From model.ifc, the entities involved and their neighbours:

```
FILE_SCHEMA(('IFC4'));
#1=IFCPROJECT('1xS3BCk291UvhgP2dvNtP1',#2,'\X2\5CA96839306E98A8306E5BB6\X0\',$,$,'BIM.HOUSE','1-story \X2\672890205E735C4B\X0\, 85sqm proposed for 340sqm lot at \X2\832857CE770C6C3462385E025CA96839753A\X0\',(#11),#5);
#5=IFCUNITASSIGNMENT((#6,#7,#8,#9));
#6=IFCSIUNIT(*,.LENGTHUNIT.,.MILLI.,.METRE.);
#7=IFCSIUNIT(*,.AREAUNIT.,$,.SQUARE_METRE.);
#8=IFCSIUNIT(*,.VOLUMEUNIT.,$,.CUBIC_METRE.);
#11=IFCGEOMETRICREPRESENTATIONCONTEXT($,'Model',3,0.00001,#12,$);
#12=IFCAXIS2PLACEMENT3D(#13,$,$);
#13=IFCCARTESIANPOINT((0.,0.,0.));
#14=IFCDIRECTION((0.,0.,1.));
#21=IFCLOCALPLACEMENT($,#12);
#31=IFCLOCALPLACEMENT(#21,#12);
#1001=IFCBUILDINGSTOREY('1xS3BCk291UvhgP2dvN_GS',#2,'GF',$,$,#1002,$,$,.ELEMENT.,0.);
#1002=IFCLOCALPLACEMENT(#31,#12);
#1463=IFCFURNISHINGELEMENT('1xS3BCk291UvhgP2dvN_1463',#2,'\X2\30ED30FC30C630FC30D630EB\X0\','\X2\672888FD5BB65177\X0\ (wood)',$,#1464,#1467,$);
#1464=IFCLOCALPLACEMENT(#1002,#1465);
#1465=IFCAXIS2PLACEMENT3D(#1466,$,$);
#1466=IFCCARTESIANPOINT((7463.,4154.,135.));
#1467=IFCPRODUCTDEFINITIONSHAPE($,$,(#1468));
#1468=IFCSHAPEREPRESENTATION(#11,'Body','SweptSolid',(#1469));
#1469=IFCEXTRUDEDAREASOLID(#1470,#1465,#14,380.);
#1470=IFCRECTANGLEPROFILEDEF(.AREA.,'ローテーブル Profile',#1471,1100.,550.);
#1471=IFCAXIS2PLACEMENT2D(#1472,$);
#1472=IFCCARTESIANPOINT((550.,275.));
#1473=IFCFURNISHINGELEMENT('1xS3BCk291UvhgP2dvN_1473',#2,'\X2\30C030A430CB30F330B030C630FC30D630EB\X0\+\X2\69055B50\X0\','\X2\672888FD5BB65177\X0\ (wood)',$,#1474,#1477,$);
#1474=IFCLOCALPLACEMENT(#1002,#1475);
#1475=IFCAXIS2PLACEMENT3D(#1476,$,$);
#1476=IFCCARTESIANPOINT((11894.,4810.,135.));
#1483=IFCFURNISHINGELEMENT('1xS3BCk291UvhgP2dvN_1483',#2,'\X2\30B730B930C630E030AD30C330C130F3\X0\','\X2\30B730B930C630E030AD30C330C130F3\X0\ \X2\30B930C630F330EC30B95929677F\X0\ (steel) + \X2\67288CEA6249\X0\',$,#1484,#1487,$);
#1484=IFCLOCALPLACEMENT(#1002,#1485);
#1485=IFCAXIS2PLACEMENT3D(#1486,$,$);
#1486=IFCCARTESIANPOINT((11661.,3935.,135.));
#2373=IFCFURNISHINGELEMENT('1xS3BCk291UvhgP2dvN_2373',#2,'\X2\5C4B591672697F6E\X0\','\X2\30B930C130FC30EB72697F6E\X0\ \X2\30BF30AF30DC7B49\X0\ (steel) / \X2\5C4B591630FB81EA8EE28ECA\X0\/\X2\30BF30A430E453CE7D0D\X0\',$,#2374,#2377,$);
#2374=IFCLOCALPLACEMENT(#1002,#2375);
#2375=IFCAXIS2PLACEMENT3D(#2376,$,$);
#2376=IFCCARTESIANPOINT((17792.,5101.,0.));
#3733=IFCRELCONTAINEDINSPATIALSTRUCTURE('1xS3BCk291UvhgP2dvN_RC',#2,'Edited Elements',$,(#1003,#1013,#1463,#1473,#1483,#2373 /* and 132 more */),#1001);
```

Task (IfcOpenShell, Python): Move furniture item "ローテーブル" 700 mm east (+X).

```python
import ifcopenshell
import ifcopenshell.api.geometry
import ifcopenshell.util.placement
import ifcopenshell.util.unit

model = ifcopenshell.open("model.ifc")
unit_scale = ifcopenshell.util.unit.calculate_unit_scale(model)

item = model.by_guid("1xS3BCk291UvhgP2dvN_1463")
matrix = ifcopenshell.util.placement.get_local_placement(item.ObjectPlacement)
matrix[0, 3] += 0.7 / unit_scale
ifcopenshell.api.geometry.edit_object_placement(model, product=item, matrix=matrix, is_si=False)

print(ifcopenshell.util.placement.get_local_placement(item.ObjectPlacement).round(3) + 0.0)

model.write("model-out.ifc")
```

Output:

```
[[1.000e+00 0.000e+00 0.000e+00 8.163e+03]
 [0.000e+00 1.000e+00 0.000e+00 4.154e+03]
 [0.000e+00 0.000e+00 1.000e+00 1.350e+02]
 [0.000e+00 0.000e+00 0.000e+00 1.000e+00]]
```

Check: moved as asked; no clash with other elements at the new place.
